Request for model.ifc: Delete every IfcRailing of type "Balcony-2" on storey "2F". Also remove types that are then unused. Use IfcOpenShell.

First a look at what the model holds.

```python
import ifcopenshell
import ifcopenshell.util.element

model = ifcopenshell.open("model.ifc")
print(model.schema)
storey = next(s for s in model.by_type("IfcBuildingStorey") if s.Name == "2F")
railings = [e for e in ifcopenshell.util.element.get_decomposition(storey) if e.is_a("IfcRailing")]
seen = {}
for e in railings:
    element_type = ifcopenshell.util.element.get_type(e)
    name = element_type.Name if element_type not in (None, e) else None
    seen[name] = seen.get(name, 0) + 1
for name, count in sorted(seen.items(), key=str):
    print(count, "x", name)
```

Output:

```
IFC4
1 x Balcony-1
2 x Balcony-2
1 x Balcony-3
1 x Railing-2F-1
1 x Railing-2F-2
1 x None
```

```python
import ifcopenshell
import ifcopenshell.api.root
import ifcopenshell.util.element

model = ifcopenshell.open("model.ifc")

storey = next(s for s in model.by_type("IfcBuildingStorey") if s.Name == "2F")
railings = [e for e in ifcopenshell.util.element.get_decomposition(storey) if e.is_a("IfcRailing")]
targets = [e for e in railings if (t := ifcopenshell.util.element.get_type(e)) not in (None, e) and t.Name == "Balcony-2"]
types = {ifcopenshell.util.element.get_type(e) for e in targets} - {None, *targets}

for e in targets:
    ifcopenshell.api.root.remove_product(model, product=e)
print(len(targets), "removed")

unused = [t for t in types if not ifcopenshell.util.element.get_types(t)]
for t in unused:
    ifcopenshell.api.root.remove_product(model, product=t)
print(len(unused), "unused types removed")

model.write("model_rev.ifc")
```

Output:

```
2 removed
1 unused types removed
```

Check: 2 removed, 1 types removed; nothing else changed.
